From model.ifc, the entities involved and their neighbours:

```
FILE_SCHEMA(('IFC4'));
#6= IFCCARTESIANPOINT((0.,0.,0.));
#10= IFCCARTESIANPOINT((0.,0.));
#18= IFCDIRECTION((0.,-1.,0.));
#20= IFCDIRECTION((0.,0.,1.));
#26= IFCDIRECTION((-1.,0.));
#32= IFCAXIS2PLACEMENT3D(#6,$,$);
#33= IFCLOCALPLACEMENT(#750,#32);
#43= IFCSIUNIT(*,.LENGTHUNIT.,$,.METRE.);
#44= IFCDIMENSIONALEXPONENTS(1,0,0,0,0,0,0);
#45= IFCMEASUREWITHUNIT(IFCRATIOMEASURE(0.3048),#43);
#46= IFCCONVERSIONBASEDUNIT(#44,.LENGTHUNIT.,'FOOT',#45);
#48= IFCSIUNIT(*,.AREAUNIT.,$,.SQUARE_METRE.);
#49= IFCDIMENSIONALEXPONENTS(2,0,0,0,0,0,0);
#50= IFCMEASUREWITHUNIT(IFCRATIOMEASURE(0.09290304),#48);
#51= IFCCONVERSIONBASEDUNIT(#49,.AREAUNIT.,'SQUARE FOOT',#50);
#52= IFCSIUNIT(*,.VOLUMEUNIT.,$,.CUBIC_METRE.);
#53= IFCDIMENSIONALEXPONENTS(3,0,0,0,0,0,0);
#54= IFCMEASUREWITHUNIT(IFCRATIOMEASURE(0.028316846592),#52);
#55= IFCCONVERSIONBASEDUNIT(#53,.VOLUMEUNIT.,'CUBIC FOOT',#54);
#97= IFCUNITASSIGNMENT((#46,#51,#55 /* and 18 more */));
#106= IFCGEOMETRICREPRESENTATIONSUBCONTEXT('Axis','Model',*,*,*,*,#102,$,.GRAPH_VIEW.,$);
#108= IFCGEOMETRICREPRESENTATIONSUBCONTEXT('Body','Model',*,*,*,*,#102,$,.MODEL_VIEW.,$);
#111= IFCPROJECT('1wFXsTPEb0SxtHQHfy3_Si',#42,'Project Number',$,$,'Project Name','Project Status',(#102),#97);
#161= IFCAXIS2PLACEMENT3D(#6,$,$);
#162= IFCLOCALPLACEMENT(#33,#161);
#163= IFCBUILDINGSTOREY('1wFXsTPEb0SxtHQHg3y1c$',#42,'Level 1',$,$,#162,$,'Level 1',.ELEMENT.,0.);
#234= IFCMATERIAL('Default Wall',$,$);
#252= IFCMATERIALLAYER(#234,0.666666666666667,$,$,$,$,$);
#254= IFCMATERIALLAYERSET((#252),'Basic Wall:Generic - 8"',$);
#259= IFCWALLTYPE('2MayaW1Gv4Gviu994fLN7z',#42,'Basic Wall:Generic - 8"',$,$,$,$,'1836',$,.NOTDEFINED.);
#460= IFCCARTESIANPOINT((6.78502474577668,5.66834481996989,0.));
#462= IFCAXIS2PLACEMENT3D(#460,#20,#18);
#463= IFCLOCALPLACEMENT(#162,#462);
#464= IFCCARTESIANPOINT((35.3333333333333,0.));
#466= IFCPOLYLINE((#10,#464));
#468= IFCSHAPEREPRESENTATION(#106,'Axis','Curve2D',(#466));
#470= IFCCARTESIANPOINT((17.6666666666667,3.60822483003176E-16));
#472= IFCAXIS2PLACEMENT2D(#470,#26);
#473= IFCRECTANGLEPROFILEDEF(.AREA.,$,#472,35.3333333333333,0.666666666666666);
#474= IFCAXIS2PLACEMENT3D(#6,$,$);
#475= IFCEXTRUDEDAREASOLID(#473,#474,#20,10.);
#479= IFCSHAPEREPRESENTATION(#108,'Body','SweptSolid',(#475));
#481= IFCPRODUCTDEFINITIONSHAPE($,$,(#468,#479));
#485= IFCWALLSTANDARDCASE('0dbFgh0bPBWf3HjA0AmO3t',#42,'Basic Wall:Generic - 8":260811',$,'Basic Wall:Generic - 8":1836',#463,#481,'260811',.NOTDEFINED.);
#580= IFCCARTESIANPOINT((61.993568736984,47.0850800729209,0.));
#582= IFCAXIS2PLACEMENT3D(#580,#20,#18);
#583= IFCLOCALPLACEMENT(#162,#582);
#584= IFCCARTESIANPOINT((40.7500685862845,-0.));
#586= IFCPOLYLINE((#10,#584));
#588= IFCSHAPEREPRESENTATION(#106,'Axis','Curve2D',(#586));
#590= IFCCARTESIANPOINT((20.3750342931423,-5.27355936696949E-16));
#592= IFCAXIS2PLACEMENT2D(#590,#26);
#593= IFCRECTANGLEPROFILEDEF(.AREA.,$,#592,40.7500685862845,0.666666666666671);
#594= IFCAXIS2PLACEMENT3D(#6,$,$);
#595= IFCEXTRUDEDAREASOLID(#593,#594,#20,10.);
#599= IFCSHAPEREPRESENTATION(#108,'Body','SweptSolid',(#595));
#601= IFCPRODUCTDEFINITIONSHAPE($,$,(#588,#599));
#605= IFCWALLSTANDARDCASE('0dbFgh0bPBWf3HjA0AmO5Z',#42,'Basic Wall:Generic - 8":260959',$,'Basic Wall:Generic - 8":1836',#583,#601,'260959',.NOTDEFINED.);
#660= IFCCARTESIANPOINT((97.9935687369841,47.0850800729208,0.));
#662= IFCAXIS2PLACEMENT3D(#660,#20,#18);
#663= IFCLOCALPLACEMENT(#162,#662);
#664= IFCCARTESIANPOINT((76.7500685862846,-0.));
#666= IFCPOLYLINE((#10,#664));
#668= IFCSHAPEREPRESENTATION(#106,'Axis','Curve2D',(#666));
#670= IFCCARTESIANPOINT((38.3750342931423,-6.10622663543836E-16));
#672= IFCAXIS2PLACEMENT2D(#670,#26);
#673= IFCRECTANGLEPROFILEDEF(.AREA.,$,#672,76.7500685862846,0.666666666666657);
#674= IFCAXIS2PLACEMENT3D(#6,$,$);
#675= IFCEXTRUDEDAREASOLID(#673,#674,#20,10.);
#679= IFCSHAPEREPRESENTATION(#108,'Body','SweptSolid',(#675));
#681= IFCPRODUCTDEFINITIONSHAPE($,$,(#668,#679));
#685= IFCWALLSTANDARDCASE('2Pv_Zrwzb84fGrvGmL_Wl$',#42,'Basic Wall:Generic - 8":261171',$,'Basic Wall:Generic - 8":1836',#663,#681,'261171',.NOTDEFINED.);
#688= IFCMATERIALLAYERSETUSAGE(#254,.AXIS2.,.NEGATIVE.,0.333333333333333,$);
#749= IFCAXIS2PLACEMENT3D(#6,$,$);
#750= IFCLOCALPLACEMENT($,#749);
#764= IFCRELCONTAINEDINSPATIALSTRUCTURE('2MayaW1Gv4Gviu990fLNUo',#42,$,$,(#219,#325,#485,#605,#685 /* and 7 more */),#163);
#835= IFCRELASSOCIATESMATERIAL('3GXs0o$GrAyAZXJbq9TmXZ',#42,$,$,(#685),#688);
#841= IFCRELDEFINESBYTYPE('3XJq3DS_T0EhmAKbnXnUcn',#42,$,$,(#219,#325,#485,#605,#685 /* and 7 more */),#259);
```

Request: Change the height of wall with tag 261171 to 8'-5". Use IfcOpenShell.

```python
import ifcopenshell
import ifcopenshell.geom
import ifcopenshell.util.representation
import ifcopenshell.util.shape
import ifcopenshell.util.unit

model = ifcopenshell.open("model.ifc")
unit_scale = ifcopenshell.util.unit.calculate_unit_scale(model)
settings = ifcopenshell.geom.settings()


def volume(element):
    """Net volume in cubic metres, openings subtracted."""
    shape = ifcopenshell.geom.create_shape(settings, element)
    return ifcopenshell.util.shape.get_volume(shape.geometry)


wall = model.by_id(685)
before = volume(wall)

body = ifcopenshell.util.representation.get_representation(wall, "Model", "Body")
solid = body.Items[0]
old_height = solid.Depth
solid.Depth = 101 * 0.0254 / unit_scale
after = volume(wall)

print(f"height {old_height:g} -> {solid.Depth:g}, volume {before:.3f} -> {after:.3f} m3")

model.write("model-out.ifc")
```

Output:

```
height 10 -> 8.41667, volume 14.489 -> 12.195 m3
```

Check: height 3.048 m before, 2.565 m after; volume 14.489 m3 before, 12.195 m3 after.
